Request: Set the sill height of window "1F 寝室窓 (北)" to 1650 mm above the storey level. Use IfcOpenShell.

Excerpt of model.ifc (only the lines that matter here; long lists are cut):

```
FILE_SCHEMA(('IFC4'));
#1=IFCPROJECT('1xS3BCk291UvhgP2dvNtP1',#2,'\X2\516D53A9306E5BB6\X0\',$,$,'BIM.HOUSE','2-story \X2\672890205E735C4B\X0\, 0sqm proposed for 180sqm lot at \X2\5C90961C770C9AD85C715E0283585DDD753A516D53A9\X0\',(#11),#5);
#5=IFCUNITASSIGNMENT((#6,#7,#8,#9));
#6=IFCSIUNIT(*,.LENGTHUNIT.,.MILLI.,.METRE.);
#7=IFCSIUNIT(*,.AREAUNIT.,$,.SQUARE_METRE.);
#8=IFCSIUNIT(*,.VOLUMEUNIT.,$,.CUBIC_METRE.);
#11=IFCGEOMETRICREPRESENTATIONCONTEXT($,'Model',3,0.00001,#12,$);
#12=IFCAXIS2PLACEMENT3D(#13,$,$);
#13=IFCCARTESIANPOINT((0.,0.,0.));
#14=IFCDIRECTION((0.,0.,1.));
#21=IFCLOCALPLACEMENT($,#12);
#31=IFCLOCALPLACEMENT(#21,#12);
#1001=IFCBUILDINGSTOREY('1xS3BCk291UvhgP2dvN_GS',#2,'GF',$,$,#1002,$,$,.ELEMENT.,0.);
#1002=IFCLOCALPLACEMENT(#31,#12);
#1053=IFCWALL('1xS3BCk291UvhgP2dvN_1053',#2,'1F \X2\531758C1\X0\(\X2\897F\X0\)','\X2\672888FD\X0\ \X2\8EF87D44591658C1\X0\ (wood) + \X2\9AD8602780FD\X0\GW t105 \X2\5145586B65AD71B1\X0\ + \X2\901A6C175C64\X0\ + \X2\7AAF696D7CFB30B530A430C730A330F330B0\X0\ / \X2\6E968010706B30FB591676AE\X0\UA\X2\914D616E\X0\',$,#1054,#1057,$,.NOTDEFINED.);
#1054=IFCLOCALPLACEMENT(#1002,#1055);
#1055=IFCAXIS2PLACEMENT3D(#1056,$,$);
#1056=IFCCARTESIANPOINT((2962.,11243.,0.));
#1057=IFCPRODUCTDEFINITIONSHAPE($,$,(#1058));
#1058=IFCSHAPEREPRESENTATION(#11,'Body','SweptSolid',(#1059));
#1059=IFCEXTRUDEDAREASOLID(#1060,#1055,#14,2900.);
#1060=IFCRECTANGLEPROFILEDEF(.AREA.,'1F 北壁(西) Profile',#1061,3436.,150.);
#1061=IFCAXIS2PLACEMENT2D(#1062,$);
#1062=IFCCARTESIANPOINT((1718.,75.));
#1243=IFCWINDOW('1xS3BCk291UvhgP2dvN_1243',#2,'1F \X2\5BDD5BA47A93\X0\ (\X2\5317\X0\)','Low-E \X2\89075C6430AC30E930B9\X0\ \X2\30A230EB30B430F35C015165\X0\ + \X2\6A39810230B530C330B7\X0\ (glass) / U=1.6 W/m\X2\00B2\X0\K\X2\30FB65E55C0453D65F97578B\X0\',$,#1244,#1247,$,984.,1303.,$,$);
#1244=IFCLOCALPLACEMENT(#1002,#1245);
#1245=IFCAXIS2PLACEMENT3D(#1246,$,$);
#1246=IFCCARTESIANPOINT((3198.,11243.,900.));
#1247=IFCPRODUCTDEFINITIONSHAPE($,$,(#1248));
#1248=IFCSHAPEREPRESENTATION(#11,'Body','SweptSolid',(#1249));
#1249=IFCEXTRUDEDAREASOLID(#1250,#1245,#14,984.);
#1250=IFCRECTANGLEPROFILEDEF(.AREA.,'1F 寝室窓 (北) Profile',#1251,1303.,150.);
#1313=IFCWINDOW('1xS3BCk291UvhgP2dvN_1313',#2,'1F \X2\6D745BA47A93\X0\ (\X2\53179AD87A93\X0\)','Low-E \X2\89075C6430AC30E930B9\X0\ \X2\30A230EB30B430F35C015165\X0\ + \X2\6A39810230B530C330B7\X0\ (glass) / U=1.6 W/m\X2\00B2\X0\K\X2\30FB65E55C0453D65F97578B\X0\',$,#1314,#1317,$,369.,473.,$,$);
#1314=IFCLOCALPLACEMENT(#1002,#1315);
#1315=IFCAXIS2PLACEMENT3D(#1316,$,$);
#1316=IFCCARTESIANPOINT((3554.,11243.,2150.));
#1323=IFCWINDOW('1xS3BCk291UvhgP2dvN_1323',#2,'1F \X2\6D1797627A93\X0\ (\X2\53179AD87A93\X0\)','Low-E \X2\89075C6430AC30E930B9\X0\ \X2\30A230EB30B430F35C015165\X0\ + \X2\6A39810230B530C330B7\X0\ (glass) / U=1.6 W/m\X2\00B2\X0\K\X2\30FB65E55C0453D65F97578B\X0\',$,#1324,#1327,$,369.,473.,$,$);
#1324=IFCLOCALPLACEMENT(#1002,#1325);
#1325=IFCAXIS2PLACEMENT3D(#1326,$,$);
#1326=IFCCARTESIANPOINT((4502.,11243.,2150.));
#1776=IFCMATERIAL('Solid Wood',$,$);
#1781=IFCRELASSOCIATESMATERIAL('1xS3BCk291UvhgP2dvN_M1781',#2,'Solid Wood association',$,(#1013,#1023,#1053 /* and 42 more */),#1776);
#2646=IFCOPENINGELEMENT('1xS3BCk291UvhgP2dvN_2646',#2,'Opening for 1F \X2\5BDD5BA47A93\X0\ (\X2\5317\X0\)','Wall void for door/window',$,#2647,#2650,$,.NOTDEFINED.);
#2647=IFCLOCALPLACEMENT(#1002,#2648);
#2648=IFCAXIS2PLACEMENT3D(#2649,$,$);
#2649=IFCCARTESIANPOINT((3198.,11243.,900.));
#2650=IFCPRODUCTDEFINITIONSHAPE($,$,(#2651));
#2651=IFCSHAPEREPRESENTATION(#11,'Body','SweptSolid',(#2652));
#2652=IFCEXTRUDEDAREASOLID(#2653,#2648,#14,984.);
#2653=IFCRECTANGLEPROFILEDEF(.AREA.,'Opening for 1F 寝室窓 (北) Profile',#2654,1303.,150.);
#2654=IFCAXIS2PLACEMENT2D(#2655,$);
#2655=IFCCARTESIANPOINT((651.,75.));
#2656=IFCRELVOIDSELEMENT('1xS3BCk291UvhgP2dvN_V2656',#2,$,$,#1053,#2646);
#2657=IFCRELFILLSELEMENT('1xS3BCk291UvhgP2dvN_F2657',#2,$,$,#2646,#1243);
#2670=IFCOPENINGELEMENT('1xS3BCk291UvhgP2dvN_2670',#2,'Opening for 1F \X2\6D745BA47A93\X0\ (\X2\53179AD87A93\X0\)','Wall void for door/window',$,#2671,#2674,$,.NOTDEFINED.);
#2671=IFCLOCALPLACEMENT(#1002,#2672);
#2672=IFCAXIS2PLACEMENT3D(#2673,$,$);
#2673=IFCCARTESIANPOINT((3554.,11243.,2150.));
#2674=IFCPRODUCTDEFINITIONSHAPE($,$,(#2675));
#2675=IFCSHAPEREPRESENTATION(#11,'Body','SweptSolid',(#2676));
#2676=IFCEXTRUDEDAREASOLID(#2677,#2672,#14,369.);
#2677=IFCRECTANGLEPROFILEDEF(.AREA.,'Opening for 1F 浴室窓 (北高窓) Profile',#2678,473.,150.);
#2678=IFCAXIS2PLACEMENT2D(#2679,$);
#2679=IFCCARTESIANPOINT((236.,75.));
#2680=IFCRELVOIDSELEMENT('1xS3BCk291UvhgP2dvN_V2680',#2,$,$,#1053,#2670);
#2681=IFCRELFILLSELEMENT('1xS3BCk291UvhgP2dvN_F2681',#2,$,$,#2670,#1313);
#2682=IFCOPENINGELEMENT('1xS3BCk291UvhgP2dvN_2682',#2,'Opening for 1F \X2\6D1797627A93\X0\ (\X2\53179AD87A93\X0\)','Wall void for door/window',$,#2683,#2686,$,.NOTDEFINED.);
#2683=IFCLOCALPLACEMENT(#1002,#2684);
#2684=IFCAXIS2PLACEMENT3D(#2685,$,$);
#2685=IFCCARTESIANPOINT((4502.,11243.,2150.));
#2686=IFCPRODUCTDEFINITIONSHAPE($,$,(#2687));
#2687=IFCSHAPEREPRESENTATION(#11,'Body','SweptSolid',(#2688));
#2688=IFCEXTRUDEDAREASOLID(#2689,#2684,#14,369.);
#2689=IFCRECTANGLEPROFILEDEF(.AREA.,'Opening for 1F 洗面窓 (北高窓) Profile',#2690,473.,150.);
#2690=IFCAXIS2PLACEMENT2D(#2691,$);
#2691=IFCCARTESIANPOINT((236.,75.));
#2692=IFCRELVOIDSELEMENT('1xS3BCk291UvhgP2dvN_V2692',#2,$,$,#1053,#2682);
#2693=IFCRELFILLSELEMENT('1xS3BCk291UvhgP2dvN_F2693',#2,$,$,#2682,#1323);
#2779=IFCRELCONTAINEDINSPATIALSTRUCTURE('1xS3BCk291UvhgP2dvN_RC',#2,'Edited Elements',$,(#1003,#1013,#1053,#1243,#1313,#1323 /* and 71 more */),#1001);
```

```python
import numpy as np
import ifcopenshell
import ifcopenshell.api.geometry
import ifcopenshell.geom
import ifcopenshell.util.element
import ifcopenshell.util.placement
import ifcopenshell.util.shape
import ifcopenshell.util.unit

model = ifcopenshell.open("model.ifc")
unit_scale = ifcopenshell.util.unit.calculate_unit_scale(model)

window = model.by_guid("1xS3BCk291UvhgP2dvN_1243")
opening = window.FillsVoids[0].RelatingOpeningElement
storey = ifcopenshell.util.element.get_container(window, ifc_class="IfcBuildingStorey")
level = ifcopenshell.util.placement.get_local_placement(storey.ObjectPlacement)[2, 3]

# The opening's origin need not be at the sill, so measure its lowest point.
shape = ifcopenshell.geom.create_shape(ifcopenshell.geom.settings(), opening)
bottom = ifcopenshell.util.shape.get_shape_bottom_elevation(shape, shape.geometry) / unit_scale
dz = level + 1.65 / unit_scale - bottom

shift = np.array([0.0, 0.0, dz])
# The window is not placed relative to its opening, so move both.
for product in (opening, window):
    matrix = ifcopenshell.util.placement.get_local_placement(product.ObjectPlacement)
    matrix[:3, 3] += shift
    ifcopenshell.api.geometry.edit_object_placement(model, product=product, matrix=matrix, is_si=False)

print(f"moved by {dz * unit_scale:+.3f} m")

model.write("model_edited.ifc")
```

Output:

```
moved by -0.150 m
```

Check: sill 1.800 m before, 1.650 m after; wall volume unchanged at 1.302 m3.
